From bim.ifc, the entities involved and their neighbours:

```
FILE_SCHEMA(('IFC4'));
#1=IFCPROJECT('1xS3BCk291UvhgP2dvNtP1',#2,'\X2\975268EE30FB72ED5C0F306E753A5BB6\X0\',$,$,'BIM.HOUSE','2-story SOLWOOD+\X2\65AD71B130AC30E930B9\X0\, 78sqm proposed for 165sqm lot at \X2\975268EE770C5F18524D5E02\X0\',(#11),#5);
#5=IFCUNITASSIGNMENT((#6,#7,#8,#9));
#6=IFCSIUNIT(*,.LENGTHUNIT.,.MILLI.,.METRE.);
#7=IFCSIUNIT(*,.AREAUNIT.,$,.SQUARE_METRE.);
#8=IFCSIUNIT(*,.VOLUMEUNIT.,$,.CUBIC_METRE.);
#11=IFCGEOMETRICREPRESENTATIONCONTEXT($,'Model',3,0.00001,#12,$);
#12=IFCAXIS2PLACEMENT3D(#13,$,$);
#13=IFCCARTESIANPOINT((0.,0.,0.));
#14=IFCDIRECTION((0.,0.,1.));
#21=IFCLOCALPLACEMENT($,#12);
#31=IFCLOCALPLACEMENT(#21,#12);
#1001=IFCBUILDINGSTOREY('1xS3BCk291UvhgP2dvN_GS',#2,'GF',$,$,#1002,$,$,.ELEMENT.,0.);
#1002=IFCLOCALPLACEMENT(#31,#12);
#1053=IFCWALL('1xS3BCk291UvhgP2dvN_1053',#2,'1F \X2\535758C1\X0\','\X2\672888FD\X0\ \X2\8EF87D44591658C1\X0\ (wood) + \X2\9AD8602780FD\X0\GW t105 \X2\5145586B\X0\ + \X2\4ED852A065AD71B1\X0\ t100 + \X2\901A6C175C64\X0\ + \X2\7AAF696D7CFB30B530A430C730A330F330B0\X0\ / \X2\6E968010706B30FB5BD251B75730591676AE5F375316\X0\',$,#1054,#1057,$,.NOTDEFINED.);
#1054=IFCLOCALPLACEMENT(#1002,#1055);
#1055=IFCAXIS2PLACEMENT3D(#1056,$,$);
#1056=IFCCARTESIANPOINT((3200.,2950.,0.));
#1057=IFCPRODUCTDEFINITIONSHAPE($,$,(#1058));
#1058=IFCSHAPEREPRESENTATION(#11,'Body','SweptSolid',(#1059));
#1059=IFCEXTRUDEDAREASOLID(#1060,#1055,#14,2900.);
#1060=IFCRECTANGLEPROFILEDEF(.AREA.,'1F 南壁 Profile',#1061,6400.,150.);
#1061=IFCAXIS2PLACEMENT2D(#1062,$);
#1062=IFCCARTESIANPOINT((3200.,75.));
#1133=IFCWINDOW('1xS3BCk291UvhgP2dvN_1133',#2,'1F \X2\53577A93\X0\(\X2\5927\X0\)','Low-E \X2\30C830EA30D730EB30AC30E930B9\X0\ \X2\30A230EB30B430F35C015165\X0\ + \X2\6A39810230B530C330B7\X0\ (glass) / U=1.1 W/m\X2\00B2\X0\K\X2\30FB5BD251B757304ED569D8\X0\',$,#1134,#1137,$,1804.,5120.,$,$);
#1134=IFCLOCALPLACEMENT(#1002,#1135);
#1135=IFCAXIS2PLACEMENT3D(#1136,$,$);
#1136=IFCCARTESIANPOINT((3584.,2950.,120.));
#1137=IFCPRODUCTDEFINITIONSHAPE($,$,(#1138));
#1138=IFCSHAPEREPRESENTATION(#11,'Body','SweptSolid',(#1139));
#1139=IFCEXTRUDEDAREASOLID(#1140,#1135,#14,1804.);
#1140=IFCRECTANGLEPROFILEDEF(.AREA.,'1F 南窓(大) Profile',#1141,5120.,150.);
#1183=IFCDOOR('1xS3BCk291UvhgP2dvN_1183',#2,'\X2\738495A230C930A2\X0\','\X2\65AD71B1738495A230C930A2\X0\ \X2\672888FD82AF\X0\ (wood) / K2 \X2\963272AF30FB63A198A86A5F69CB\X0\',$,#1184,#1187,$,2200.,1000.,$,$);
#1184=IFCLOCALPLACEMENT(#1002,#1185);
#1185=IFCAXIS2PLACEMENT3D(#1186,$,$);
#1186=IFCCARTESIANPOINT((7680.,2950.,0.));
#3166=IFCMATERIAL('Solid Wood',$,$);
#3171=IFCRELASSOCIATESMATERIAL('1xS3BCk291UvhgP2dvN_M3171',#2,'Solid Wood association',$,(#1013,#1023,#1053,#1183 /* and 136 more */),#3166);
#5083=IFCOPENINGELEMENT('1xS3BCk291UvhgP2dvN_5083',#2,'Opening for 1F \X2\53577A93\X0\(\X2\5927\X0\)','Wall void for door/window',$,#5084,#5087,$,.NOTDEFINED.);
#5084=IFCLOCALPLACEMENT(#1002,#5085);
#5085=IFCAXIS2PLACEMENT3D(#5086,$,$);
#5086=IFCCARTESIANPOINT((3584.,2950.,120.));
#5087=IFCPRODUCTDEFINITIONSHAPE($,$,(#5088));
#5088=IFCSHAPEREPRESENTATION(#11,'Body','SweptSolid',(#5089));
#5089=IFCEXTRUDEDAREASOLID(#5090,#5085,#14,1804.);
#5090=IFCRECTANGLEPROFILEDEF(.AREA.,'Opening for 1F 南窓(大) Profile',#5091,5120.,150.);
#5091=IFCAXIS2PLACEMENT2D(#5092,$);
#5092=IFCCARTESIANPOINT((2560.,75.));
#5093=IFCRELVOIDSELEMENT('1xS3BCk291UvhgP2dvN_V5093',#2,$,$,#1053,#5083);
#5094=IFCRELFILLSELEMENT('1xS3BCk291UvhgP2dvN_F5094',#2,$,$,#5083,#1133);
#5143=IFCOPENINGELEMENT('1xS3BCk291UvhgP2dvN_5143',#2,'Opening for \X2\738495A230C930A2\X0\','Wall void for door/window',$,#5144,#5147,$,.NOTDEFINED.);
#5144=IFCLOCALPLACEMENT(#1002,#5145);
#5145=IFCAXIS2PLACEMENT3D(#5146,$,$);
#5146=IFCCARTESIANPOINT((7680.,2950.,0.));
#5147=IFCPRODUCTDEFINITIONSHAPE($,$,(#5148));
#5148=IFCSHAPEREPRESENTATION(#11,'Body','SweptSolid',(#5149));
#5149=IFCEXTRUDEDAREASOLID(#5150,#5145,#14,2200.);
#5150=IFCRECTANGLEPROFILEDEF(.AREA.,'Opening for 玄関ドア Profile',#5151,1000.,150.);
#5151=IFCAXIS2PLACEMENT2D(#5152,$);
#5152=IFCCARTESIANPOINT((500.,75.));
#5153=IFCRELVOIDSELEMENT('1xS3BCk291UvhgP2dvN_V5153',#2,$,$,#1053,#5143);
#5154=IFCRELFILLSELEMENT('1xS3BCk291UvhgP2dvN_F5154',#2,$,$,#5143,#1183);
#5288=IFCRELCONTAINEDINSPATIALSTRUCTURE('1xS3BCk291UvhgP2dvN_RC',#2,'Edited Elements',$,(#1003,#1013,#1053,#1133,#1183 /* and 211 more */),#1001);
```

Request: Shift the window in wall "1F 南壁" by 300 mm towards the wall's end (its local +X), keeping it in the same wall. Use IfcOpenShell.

```python
import ifcopenshell
import ifcopenshell.api.geometry
import ifcopenshell.util.placement
import ifcopenshell.util.unit

model = ifcopenshell.open("bim.ifc")
unit_scale = ifcopenshell.util.unit.calculate_unit_scale(model)

window = model.by_guid("1xS3BCk291UvhgP2dvN_1133")
opening = window.FillsVoids[0].RelatingOpeningElement
wall = opening.VoidsElements[0].RelatingBuildingElement

wall_matrix = ifcopenshell.util.placement.get_local_placement(wall.ObjectPlacement)
shift = wall_matrix[:3, 0] * 0.3 / unit_scale
before = ifcopenshell.util.placement.get_local_placement(window.ObjectPlacement)[:3, 3].copy()

# The window is not placed relative to its opening, so move both.
for product in (opening, window):
    matrix = ifcopenshell.util.placement.get_local_placement(product.ObjectPlacement)
    matrix[:3, 3] += shift
    ifcopenshell.api.geometry.edit_object_placement(model, product=product, matrix=matrix, is_si=False)

after = ifcopenshell.util.placement.get_local_placement(window.ObjectPlacement)[:3, 3]
print("window moved by", (after - before).round(3) + 0.0)

model.write("bim_rev.ifc")
```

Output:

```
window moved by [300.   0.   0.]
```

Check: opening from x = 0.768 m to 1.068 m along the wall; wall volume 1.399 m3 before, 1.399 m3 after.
